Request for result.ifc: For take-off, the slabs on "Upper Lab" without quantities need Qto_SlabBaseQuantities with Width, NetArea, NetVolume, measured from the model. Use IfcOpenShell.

First a look at what the model holds.

```python
import ifcopenshell
import ifcopenshell.util.element
import ifcopenshell.util.unit

model = ifcopenshell.open("result.ifc")
print(model.schema)
for unit_type in ("LENGTHUNIT", "AREAUNIT", "VOLUMEUNIT"):
    print(unit_type, ifcopenshell.util.unit.calculate_unit_scale(model, unit_type))
storey = next(s for s in model.by_type("IfcBuildingStorey") if s.Name == "Upper Lab")
slabs = [e for e in ifcopenshell.util.element.get_decomposition(storey) if e.is_a("IfcSlab")]
for e in sorted(slabs, key=lambda e: e.id()):
    print(e.id(), e.is_a(), e.Name, list(ifcopenshell.util.element.get_psets(e, qtos_only=True)), sep=" | ")
```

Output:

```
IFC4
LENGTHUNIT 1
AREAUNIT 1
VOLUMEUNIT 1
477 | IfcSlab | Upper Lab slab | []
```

```python
import ifcopenshell
import ifcopenshell.api.pset
import ifcopenshell.geom
import ifcopenshell.util.element
import ifcopenshell.util.shape
import ifcopenshell.util.unit

model = ifcopenshell.open("result.ifc")
unit_scale = ifcopenshell.util.unit.calculate_unit_scale(model)
area_scale = ifcopenshell.util.unit.calculate_unit_scale(model, "AREAUNIT")
volume_scale = ifcopenshell.util.unit.calculate_unit_scale(model, "VOLUMEUNIT")
settings = ifcopenshell.geom.settings()

storey = next(s for s in model.by_type("IfcBuildingStorey") if s.Name == "Upper Lab")
slabs = [e for e in ifcopenshell.util.element.get_decomposition(storey) if e.is_a("IfcSlab")]

for e in sorted(slabs, key=lambda e: e.id()):
    if ifcopenshell.util.element.get_psets(e, qtos_only=True, should_inherit=False):
        continue
    # Geometry comes back in metres, in the element's own axes.
    shape = ifcopenshell.geom.create_shape(settings, e)
    values = {
        "Width": ifcopenshell.util.shape.get_z(shape.geometry) / unit_scale,
        "NetArea": ifcopenshell.util.shape.get_footprint_area(shape.geometry) / area_scale,
        "NetVolume": ifcopenshell.util.shape.get_volume(shape.geometry) / volume_scale,
    }
    qto = ifcopenshell.api.pset.add_qto(model, product=e, name="Qto_SlabBaseQuantities")
    ifcopenshell.api.pset.edit_qto(model, qto=qto, properties=values)
    print(e.id(), {k: round(v, 3) for k, v in values.items()})

model.write("result_rev.ifc")
```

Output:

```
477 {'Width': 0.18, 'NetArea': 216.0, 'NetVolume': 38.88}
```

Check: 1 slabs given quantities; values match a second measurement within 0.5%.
